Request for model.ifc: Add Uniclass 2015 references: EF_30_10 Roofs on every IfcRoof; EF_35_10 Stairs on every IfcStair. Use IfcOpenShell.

First a look at what the model holds.

```python
import ifcopenshell

model = ifcopenshell.open("model.ifc")
print(model.schema)
print("classifications:", [c.Name for c in model.by_type("IfcClassification")])
for ifc_class in ("IfcDoor", "IfcRoof", "IfcStair", "IfcWall", "IfcWindow"):
    print(ifc_class, len(model.by_type(ifc_class)))
```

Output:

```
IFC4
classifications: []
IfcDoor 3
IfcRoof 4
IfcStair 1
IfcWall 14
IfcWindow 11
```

```python
import ifcopenshell
import ifcopenshell.api.classification

model = ifcopenshell.open("model.ifc")

system = ifcopenshell.api.classification.add_classification(model, classification="Uniclass 2015")

codes = {
    "IfcRoof": ("EF_30_10", "Roofs"),
    "IfcStair": ("EF_35_10", "Stairs"),
}
for ifc_class, (code, name) in codes.items():
    products = model.by_type(ifc_class)
    ifcopenshell.api.classification.add_reference(
        model, products=products, classification=system, identification=code, name=name
    )
    print(code, len(products))

model.write("model_rev.ifc")
```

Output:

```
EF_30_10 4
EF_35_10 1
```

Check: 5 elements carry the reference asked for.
